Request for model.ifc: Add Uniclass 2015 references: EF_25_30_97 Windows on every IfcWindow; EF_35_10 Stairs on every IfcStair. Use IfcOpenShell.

First a look at what the model holds.

```python
import ifcopenshell

model = ifcopenshell.open("model.ifc")
print(model.schema)
print("classifications:", [c.Name for c in model.by_type("IfcClassification")])
for ifc_class in ("IfcDoor", "IfcRoof", "IfcStair", "IfcWall", "IfcWindow"):
    print(ifc_class, len(model.by_type(ifc_class)))
```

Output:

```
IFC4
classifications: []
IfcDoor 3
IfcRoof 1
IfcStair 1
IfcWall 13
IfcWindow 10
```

```python
import ifcopenshell
import ifcopenshell.api.classification

model = ifcopenshell.open("model.ifc")

system = ifcopenshell.api.classification.add_classification(model, classification="Uniclass 2015")

codes = {
    "IfcWindow": ("EF_25_30_97", "Windows"),
    "IfcStair": ("EF_35_10", "Stairs"),
}
for ifc_class, (code, name) in codes.items():
    products = model.by_type(ifc_class)
    ifcopenshell.api.classification.add_reference(
        model, products=products, classification=system, identification=code, name=name
    )
    print(code, len(products))

model.write("model_edited.ifc")
```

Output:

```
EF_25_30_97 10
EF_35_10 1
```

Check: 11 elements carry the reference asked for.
